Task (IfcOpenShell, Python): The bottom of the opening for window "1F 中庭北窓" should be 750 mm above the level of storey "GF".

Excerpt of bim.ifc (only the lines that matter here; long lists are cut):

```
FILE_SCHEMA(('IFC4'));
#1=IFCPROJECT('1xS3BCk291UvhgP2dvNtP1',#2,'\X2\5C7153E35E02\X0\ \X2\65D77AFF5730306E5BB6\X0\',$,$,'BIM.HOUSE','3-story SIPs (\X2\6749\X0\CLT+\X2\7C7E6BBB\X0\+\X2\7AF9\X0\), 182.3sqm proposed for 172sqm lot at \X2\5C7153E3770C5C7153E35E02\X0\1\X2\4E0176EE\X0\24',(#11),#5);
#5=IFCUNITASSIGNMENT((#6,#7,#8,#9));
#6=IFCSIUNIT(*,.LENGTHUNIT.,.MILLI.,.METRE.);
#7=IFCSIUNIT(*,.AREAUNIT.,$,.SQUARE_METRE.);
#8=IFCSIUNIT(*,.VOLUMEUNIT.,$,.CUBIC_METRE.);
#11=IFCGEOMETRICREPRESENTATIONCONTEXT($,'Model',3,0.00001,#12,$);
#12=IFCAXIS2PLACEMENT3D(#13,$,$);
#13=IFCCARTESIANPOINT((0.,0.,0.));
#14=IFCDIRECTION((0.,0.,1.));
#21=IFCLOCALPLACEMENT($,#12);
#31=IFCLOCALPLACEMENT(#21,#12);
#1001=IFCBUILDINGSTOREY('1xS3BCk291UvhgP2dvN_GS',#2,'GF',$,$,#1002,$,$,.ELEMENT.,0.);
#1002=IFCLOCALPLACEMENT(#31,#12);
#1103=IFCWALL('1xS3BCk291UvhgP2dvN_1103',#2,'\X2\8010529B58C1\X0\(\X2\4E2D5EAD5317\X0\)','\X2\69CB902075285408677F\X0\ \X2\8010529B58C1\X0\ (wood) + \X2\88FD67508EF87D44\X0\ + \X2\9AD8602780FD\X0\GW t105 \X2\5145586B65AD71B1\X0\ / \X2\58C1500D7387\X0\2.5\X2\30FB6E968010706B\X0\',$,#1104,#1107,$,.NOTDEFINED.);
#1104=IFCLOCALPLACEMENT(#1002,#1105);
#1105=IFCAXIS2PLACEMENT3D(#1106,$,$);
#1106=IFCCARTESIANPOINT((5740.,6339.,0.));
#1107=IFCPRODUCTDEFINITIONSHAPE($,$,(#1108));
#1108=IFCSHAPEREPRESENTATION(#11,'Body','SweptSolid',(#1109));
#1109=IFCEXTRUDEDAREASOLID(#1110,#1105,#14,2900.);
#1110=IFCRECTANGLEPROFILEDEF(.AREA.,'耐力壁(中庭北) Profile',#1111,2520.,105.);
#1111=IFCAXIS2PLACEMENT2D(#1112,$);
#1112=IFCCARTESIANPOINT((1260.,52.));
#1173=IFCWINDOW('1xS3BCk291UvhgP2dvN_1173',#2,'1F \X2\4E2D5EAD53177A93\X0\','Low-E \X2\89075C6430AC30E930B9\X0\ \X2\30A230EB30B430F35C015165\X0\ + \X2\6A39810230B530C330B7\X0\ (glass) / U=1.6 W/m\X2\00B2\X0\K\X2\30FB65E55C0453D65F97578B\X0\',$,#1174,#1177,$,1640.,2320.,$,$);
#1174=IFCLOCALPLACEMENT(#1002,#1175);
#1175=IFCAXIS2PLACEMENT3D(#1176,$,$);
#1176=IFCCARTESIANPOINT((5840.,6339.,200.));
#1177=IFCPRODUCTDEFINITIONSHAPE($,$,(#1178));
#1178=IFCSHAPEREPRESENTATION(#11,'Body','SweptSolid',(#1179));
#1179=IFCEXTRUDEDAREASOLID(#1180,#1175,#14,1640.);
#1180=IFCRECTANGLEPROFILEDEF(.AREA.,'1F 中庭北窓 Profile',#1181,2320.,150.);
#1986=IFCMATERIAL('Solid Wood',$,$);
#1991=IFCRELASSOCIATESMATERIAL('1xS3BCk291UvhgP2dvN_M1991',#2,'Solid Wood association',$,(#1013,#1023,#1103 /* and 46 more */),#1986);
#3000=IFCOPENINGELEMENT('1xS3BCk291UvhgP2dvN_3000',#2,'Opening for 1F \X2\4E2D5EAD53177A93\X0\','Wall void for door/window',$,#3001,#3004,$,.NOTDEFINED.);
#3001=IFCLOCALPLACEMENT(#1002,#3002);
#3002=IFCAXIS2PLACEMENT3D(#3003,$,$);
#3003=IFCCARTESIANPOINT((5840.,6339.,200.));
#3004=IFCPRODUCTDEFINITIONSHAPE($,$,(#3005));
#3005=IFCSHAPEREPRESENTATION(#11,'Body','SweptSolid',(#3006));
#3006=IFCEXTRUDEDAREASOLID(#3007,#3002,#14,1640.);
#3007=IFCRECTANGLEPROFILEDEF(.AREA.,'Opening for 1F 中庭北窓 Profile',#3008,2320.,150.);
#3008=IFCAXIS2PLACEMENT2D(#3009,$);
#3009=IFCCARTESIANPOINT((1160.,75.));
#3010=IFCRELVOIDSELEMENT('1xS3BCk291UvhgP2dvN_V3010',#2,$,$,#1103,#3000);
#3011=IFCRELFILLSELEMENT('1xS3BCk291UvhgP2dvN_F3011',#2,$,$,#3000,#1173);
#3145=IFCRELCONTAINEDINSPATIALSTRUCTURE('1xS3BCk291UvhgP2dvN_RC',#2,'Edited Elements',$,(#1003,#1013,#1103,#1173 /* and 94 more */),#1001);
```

```python
import numpy as np
import ifcopenshell
import ifcopenshell.api.geometry
import ifcopenshell.geom
import ifcopenshell.util.element
import ifcopenshell.util.placement
import ifcopenshell.util.shape
import ifcopenshell.util.unit

model = ifcopenshell.open("bim.ifc")
unit_scale = ifcopenshell.util.unit.calculate_unit_scale(model)

window = model.by_guid("1xS3BCk291UvhgP2dvN_1173")
opening = window.FillsVoids[0].RelatingOpeningElement
storey = ifcopenshell.util.element.get_container(window, ifc_class="IfcBuildingStorey")
level = ifcopenshell.util.placement.get_local_placement(storey.ObjectPlacement)[2, 3]

# The opening's origin need not be at the sill, so measure its lowest point.
shape = ifcopenshell.geom.create_shape(ifcopenshell.geom.settings(), opening)
bottom = ifcopenshell.util.shape.get_shape_bottom_elevation(shape, shape.geometry) / unit_scale
dz = level + 750.0 - bottom

shift = np.array([0.0, 0.0, dz])
# The window is not placed relative to its opening, so move both.
for product in (opening, window):
    matrix = ifcopenshell.util.placement.get_local_placement(product.ObjectPlacement)
    matrix[:3, 3] += shift
    ifcopenshell.api.geometry.edit_object_placement(model, product=product, matrix=matrix, is_si=False)

print(f"moved by {dz * unit_scale:+.3f} m")

model.write("bim_v2.ifc")
```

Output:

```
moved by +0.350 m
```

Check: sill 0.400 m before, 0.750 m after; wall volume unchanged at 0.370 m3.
